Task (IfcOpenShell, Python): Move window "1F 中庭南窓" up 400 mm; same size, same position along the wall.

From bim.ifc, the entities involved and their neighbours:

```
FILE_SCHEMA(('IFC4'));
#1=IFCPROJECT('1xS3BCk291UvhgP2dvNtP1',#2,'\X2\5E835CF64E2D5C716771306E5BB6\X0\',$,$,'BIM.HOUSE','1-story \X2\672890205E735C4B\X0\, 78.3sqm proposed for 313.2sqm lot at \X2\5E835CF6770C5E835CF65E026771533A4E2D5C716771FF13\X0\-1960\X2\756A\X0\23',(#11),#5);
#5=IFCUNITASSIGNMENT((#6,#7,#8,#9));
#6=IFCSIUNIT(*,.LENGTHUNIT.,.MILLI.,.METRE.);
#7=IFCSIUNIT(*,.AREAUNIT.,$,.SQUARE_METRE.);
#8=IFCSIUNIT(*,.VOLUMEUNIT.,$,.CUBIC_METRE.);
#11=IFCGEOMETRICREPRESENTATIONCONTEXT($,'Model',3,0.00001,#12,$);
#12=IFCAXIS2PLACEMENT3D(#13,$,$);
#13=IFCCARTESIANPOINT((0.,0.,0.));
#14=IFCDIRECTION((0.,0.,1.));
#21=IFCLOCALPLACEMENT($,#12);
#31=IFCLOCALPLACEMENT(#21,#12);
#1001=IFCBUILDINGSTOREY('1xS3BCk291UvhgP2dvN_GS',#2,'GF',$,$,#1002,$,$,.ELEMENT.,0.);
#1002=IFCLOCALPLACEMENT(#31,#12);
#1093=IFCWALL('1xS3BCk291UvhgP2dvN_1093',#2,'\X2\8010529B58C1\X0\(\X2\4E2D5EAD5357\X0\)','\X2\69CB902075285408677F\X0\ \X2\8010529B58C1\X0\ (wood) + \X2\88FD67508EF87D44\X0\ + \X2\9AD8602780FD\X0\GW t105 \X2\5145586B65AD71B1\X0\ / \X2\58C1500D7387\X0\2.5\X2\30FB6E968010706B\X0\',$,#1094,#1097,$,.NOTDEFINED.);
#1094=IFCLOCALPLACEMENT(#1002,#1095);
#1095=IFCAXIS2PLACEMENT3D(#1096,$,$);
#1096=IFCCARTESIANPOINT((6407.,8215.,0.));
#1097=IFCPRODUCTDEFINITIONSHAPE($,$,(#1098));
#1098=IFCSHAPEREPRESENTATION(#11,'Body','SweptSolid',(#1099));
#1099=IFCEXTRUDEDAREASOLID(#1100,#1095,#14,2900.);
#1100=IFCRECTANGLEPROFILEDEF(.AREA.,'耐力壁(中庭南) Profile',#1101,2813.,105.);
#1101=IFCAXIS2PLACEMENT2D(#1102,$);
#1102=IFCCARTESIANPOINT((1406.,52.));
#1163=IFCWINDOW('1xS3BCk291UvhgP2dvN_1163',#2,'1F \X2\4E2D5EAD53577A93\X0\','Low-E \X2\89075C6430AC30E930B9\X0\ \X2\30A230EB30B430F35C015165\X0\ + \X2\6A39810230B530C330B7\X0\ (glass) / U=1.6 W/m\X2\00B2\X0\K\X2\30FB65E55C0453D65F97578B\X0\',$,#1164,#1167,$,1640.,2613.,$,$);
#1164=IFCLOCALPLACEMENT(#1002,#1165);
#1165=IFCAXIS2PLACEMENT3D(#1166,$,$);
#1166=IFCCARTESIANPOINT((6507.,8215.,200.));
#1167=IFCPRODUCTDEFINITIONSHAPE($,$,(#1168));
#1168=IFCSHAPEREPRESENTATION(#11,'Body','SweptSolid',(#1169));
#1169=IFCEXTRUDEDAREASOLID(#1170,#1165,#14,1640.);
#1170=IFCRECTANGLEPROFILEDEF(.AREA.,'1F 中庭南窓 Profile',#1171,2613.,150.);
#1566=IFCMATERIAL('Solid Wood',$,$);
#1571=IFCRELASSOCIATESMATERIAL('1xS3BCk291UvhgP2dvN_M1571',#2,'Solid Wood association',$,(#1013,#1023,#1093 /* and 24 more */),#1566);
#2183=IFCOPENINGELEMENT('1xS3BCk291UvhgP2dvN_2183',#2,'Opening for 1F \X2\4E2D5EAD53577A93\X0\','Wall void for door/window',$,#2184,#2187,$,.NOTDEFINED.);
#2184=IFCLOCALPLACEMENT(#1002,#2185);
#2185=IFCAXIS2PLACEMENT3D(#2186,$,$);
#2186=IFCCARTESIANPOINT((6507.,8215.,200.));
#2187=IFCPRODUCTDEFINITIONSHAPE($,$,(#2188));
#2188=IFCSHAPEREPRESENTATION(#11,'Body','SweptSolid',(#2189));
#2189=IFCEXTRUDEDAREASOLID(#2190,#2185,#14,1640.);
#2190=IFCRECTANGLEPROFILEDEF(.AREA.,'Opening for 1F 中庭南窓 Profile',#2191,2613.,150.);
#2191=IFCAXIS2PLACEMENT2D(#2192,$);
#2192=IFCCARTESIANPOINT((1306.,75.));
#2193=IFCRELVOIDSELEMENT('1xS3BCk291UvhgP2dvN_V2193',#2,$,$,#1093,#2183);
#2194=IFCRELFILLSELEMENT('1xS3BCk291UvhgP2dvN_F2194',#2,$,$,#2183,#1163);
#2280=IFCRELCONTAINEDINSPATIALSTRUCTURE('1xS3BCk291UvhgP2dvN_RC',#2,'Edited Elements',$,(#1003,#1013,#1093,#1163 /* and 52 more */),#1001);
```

```python
import numpy as np
import ifcopenshell
import ifcopenshell.api.geometry
import ifcopenshell.util.placement
import ifcopenshell.util.unit

model = ifcopenshell.open("bim.ifc")
unit_scale = ifcopenshell.util.unit.calculate_unit_scale(model)

window = model.by_id(1163)
opening = window.FillsVoids[0].RelatingOpeningElement
dz = 0.4 / unit_scale

shift = np.array([0.0, 0.0, dz])
# The window is not placed relative to its opening, so move both.
for product in (opening, window):
    matrix = ifcopenshell.util.placement.get_local_placement(product.ObjectPlacement)
    matrix[:3, 3] += shift
    ifcopenshell.api.geometry.edit_object_placement(model, product=product, matrix=matrix, is_si=False)

print(f"moved by {dz * unit_scale:+.3f} m")

model.write("bim_updated.ifc")
```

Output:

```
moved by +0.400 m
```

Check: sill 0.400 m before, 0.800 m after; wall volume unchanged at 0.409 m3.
